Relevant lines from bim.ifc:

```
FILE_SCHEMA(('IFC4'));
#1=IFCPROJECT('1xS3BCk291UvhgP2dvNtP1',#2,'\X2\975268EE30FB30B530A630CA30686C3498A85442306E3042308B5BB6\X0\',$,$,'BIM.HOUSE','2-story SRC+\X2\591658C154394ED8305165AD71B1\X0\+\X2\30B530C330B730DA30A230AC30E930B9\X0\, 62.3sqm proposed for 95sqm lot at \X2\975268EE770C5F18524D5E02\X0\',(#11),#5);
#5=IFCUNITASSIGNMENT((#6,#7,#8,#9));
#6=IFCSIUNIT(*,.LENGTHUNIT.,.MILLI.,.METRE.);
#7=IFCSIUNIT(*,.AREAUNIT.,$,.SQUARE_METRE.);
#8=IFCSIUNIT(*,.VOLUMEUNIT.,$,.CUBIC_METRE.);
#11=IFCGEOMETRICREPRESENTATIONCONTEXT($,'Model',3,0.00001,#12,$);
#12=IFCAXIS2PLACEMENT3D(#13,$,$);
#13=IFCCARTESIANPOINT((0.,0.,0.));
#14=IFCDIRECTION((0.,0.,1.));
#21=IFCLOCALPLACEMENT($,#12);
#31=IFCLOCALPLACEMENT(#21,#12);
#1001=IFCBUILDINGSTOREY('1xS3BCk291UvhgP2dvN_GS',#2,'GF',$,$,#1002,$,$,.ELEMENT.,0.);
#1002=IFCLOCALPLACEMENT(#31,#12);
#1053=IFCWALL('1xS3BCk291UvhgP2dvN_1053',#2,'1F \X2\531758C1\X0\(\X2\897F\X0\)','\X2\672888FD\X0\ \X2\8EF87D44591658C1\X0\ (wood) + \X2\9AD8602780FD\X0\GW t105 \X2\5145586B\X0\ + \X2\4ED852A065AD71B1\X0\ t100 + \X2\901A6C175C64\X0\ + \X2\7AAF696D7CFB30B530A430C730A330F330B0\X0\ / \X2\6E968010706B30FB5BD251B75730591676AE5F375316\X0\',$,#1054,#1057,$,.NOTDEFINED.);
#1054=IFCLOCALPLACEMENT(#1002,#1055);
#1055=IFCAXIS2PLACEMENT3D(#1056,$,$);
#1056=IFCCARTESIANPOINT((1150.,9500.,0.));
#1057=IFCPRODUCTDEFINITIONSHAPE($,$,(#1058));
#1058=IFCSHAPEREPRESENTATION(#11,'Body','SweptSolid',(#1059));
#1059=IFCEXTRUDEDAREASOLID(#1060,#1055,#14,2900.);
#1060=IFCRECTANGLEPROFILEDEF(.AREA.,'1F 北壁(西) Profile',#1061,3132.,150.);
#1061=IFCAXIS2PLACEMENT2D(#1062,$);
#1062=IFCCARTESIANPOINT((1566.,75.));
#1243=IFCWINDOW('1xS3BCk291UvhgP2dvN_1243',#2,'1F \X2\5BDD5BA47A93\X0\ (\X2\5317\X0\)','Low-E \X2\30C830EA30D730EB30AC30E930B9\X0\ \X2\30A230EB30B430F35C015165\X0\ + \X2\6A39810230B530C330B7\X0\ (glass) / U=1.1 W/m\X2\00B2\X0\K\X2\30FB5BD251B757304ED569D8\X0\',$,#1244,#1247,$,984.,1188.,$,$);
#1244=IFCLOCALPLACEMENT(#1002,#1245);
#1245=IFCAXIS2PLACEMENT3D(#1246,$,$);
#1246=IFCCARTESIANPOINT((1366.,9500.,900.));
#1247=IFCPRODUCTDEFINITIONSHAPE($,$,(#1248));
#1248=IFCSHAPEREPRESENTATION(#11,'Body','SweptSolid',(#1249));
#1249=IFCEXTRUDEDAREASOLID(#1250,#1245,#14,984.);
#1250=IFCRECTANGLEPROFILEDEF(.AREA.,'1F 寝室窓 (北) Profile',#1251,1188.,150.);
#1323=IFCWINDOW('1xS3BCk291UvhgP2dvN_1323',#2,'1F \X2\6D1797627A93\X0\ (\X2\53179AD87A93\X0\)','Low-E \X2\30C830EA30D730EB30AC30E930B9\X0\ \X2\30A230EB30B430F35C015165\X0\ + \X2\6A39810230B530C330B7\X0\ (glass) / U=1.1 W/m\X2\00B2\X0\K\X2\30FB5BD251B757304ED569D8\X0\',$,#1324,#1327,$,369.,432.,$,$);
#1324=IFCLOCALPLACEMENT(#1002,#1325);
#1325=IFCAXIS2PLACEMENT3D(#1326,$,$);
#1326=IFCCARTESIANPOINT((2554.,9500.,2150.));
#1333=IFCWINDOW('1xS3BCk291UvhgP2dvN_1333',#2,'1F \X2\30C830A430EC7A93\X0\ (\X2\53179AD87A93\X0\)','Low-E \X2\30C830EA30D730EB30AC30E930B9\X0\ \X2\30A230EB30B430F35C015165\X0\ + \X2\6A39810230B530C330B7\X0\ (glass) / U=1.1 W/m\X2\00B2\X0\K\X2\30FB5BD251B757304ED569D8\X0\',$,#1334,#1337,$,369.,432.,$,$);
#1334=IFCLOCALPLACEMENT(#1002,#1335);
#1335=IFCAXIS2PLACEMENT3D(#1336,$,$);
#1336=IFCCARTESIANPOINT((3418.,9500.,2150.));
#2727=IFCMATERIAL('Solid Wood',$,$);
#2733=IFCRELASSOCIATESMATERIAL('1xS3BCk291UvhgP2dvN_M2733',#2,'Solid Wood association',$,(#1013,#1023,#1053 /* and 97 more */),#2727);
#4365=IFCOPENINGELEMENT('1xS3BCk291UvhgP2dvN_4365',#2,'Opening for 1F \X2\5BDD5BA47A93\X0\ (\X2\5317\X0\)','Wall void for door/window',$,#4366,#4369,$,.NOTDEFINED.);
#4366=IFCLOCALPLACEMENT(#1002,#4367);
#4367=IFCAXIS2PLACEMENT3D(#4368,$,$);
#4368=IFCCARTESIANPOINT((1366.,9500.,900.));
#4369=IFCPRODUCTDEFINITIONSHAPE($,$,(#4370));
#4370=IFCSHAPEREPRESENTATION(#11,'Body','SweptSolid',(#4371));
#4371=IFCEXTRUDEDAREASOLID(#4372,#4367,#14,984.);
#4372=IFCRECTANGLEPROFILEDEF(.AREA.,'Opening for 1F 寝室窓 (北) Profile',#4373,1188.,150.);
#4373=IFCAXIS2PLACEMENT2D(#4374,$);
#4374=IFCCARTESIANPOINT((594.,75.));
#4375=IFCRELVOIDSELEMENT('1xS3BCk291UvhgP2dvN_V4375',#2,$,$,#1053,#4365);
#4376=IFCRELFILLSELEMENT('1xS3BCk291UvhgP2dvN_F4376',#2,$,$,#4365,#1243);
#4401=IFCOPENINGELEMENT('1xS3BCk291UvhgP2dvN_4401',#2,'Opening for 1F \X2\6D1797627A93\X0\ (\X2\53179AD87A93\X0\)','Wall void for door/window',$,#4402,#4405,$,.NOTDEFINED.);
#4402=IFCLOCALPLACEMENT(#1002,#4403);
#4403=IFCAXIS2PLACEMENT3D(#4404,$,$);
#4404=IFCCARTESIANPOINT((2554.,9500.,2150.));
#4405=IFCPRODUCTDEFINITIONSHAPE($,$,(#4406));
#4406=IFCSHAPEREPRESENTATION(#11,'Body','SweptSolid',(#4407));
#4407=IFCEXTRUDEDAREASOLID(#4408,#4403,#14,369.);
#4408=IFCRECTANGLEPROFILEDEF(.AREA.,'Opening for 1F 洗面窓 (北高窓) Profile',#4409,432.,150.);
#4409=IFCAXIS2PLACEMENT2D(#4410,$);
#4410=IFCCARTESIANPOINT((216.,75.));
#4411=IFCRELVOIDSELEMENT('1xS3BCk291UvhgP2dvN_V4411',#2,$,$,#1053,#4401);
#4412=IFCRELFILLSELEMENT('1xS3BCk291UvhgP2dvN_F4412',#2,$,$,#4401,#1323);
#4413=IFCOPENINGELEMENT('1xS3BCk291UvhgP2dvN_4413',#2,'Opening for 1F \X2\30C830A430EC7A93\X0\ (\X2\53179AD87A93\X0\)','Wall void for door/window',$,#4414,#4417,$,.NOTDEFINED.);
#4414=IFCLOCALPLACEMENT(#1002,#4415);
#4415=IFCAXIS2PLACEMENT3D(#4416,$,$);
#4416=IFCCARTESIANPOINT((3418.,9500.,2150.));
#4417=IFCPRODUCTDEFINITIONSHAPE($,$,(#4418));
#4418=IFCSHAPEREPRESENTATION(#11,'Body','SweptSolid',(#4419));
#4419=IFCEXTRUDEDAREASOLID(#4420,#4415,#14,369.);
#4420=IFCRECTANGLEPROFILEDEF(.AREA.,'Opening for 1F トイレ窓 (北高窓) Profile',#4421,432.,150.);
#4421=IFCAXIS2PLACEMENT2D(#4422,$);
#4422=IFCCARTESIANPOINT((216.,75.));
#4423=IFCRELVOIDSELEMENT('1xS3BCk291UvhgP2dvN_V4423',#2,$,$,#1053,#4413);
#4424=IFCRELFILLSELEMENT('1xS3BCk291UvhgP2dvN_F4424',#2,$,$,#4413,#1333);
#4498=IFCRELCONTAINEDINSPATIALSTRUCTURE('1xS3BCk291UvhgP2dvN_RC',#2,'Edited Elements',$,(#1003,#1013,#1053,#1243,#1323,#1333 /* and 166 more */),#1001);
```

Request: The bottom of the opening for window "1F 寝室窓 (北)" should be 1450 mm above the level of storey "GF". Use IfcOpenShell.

```python
import numpy as np
import ifcopenshell
import ifcopenshell.api.geometry
import ifcopenshell.geom
import ifcopenshell.util.element
import ifcopenshell.util.placement
import ifcopenshell.util.shape
import ifcopenshell.util.unit

model = ifcopenshell.open("bim.ifc")
unit_scale = ifcopenshell.util.unit.calculate_unit_scale(model)

window = model.by_guid("1xS3BCk291UvhgP2dvN_1243")
opening = window.FillsVoids[0].RelatingOpeningElement
storey = ifcopenshell.util.element.get_container(window, ifc_class="IfcBuildingStorey")
level = ifcopenshell.util.placement.get_local_placement(storey.ObjectPlacement)[2, 3]

# The opening's origin need not be at the sill, so measure its lowest point.
shape = ifcopenshell.geom.create_shape(ifcopenshell.geom.settings(), opening)
bottom = ifcopenshell.util.shape.get_shape_bottom_elevation(shape, shape.geometry) / unit_scale
dz = level + 1.45 / unit_scale - bottom

shift = np.array([0.0, 0.0, dz])
# The window is not placed relative to its opening, so move both.
for product in (opening, window):
    matrix = ifcopenshell.util.placement.get_local_placement(product.ObjectPlacement)
    matrix[:3, 3] += shift
    ifcopenshell.api.geometry.edit_object_placement(model, product=product, matrix=matrix, is_si=False)

print(f"moved by {dz * unit_scale:+.3f} m")

model.write("bim_rev.ifc")
```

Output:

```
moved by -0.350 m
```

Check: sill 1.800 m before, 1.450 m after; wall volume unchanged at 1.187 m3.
